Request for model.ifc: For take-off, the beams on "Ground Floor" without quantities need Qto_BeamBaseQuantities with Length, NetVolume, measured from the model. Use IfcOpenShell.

First a look at what the model holds.

```python
import ifcopenshell
import ifcopenshell.util.element
import ifcopenshell.util.unit

model = ifcopenshell.open("model.ifc")
print(model.schema)
for unit_type in ("LENGTHUNIT", "AREAUNIT", "VOLUMEUNIT"):
    print(unit_type, ifcopenshell.util.unit.calculate_unit_scale(model, unit_type))
storey = next(s for s in model.by_type("IfcBuildingStorey") if s.Name == "Ground Floor")
beams = [e for e in ifcopenshell.util.element.get_decomposition(storey) if e.is_a("IfcBeam")]
for e in sorted(beams, key=lambda e: e.id()):
    print(e.id(), e.is_a(), e.Name, list(ifcopenshell.util.element.get_psets(e, qtos_only=True)), sep=" | ")
```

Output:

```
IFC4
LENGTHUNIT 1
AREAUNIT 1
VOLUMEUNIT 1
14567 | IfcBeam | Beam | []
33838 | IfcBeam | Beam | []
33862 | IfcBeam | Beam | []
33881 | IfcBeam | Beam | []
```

```python
import ifcopenshell
import ifcopenshell.api.pset
import ifcopenshell.geom
import ifcopenshell.util.element
import ifcopenshell.util.shape
import ifcopenshell.util.unit

model = ifcopenshell.open("model.ifc")
unit_scale = ifcopenshell.util.unit.calculate_unit_scale(model)
volume_scale = ifcopenshell.util.unit.calculate_unit_scale(model, "VOLUMEUNIT")
settings = ifcopenshell.geom.settings()

storey = next(s for s in model.by_type("IfcBuildingStorey") if s.Name == "Ground Floor")
beams = [e for e in ifcopenshell.util.element.get_decomposition(storey) if e.is_a("IfcBeam")]

for e in sorted(beams, key=lambda e: e.id()):
    if ifcopenshell.util.element.get_psets(e, qtos_only=True, should_inherit=False):
        continue
    # Geometry comes back in metres, in the element's own axes.
    shape = ifcopenshell.geom.create_shape(settings, e)
    values = {
        "Length": ifcopenshell.util.shape.get_max_xyz(shape.geometry) / unit_scale,
        "NetVolume": ifcopenshell.util.shape.get_volume(shape.geometry) / volume_scale,
    }
    qto = ifcopenshell.api.pset.add_qto(model, product=e, name="Qto_BeamBaseQuantities")
    ifcopenshell.api.pset.edit_qto(model, qto=qto, properties=values)
    print(e.id(), {k: round(v, 3) for k, v in values.items()})

model.write("model-out.ifc")
```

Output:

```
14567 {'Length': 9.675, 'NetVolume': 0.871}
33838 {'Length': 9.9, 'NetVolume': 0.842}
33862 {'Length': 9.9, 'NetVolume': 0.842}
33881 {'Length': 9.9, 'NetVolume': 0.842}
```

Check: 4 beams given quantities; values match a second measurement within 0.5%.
